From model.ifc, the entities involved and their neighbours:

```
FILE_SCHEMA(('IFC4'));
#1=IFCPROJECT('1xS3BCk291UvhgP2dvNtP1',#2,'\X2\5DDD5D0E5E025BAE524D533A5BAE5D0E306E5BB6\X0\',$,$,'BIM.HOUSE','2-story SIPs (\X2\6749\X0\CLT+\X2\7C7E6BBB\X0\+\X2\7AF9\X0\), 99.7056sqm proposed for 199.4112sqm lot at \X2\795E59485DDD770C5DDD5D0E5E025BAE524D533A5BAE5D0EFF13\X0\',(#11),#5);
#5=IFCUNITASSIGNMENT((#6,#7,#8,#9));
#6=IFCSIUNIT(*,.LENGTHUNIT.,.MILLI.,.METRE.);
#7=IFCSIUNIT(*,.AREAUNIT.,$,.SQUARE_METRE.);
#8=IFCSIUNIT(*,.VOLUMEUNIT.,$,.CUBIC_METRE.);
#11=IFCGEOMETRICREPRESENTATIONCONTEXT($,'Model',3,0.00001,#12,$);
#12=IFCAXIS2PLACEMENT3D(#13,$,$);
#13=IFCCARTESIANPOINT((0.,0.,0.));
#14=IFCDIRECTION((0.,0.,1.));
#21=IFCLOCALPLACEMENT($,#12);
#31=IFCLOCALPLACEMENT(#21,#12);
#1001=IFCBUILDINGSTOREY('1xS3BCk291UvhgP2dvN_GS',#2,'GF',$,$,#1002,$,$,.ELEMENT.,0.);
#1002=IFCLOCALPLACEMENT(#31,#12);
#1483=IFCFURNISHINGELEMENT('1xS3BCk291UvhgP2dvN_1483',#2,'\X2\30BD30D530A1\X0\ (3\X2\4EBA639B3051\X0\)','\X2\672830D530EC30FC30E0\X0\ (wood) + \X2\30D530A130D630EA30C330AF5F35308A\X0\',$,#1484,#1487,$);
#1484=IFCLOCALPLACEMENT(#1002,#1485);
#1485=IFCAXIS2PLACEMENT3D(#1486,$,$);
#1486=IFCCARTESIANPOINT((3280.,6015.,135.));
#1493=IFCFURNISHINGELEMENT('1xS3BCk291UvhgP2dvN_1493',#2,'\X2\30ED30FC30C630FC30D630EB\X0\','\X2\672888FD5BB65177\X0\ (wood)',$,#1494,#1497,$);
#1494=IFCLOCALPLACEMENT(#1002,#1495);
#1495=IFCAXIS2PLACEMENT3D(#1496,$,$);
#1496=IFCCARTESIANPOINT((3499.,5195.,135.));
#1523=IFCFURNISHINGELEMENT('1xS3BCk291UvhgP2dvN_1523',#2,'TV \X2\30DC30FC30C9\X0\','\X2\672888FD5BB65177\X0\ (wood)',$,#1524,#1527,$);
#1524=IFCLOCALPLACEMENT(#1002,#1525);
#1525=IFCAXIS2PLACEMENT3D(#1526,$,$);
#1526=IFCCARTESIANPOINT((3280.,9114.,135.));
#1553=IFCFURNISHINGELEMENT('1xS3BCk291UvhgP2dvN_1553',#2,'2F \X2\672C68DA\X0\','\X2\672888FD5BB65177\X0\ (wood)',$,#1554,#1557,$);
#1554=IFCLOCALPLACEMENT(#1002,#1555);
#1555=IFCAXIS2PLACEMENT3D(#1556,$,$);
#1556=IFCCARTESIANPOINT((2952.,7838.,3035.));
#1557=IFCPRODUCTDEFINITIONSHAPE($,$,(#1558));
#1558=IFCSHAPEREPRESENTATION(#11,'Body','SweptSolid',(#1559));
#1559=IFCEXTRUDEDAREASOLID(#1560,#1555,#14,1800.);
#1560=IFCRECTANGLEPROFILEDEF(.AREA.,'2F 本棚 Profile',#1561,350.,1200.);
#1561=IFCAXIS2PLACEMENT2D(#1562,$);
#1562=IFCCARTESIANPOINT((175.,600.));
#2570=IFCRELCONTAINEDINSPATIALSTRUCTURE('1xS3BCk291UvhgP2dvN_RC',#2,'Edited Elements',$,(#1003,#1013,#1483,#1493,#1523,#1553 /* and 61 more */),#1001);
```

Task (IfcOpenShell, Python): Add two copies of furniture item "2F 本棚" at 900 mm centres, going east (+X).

```python
import numpy as np
import ifcopenshell
import ifcopenshell.api.geometry
import ifcopenshell.api.root
import ifcopenshell.util.element
import ifcopenshell.util.placement

model = ifcopenshell.open("model.ifc")


def reuse_history(source, copy):
    """copy_class also copies each property set's owner history, people and application; keep the originals."""
    for rel in copy.IsDefinedBy:
        if rel.is_a("IfcRelDefinesByProperties") and (history := rel.RelatingPropertyDefinition.OwnerHistory):
            rel.RelatingPropertyDefinition.OwnerHistory = source.OwnerHistory
            ifcopenshell.util.element.remove_deep2(model, history)


source = model.by_id(1553)
base = ifcopenshell.util.placement.get_local_placement(source.ObjectPlacement)
step = np.array([1.0, 0.0, 0.0]) * 900.0

for i in range(1, 3):
    copy = ifcopenshell.api.root.copy_class(model, product=source)
    copy.Representation = ifcopenshell.util.element.copy_deep(
        model, source.Representation, exclude=["IfcGeometricRepresentationContext", "IfcRepresentationMap"]
    )
    reuse_history(source, copy)
    matrix = base.copy()
    matrix[:3, 3] += i * step
    print("added at", matrix[:3, 3].round(3) + 0.0)
    ifcopenshell.api.geometry.edit_object_placement(model, product=copy, matrix=matrix, is_si=False)

model.write("model_v2.ifc")
```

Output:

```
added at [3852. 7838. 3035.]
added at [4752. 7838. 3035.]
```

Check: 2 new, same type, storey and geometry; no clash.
